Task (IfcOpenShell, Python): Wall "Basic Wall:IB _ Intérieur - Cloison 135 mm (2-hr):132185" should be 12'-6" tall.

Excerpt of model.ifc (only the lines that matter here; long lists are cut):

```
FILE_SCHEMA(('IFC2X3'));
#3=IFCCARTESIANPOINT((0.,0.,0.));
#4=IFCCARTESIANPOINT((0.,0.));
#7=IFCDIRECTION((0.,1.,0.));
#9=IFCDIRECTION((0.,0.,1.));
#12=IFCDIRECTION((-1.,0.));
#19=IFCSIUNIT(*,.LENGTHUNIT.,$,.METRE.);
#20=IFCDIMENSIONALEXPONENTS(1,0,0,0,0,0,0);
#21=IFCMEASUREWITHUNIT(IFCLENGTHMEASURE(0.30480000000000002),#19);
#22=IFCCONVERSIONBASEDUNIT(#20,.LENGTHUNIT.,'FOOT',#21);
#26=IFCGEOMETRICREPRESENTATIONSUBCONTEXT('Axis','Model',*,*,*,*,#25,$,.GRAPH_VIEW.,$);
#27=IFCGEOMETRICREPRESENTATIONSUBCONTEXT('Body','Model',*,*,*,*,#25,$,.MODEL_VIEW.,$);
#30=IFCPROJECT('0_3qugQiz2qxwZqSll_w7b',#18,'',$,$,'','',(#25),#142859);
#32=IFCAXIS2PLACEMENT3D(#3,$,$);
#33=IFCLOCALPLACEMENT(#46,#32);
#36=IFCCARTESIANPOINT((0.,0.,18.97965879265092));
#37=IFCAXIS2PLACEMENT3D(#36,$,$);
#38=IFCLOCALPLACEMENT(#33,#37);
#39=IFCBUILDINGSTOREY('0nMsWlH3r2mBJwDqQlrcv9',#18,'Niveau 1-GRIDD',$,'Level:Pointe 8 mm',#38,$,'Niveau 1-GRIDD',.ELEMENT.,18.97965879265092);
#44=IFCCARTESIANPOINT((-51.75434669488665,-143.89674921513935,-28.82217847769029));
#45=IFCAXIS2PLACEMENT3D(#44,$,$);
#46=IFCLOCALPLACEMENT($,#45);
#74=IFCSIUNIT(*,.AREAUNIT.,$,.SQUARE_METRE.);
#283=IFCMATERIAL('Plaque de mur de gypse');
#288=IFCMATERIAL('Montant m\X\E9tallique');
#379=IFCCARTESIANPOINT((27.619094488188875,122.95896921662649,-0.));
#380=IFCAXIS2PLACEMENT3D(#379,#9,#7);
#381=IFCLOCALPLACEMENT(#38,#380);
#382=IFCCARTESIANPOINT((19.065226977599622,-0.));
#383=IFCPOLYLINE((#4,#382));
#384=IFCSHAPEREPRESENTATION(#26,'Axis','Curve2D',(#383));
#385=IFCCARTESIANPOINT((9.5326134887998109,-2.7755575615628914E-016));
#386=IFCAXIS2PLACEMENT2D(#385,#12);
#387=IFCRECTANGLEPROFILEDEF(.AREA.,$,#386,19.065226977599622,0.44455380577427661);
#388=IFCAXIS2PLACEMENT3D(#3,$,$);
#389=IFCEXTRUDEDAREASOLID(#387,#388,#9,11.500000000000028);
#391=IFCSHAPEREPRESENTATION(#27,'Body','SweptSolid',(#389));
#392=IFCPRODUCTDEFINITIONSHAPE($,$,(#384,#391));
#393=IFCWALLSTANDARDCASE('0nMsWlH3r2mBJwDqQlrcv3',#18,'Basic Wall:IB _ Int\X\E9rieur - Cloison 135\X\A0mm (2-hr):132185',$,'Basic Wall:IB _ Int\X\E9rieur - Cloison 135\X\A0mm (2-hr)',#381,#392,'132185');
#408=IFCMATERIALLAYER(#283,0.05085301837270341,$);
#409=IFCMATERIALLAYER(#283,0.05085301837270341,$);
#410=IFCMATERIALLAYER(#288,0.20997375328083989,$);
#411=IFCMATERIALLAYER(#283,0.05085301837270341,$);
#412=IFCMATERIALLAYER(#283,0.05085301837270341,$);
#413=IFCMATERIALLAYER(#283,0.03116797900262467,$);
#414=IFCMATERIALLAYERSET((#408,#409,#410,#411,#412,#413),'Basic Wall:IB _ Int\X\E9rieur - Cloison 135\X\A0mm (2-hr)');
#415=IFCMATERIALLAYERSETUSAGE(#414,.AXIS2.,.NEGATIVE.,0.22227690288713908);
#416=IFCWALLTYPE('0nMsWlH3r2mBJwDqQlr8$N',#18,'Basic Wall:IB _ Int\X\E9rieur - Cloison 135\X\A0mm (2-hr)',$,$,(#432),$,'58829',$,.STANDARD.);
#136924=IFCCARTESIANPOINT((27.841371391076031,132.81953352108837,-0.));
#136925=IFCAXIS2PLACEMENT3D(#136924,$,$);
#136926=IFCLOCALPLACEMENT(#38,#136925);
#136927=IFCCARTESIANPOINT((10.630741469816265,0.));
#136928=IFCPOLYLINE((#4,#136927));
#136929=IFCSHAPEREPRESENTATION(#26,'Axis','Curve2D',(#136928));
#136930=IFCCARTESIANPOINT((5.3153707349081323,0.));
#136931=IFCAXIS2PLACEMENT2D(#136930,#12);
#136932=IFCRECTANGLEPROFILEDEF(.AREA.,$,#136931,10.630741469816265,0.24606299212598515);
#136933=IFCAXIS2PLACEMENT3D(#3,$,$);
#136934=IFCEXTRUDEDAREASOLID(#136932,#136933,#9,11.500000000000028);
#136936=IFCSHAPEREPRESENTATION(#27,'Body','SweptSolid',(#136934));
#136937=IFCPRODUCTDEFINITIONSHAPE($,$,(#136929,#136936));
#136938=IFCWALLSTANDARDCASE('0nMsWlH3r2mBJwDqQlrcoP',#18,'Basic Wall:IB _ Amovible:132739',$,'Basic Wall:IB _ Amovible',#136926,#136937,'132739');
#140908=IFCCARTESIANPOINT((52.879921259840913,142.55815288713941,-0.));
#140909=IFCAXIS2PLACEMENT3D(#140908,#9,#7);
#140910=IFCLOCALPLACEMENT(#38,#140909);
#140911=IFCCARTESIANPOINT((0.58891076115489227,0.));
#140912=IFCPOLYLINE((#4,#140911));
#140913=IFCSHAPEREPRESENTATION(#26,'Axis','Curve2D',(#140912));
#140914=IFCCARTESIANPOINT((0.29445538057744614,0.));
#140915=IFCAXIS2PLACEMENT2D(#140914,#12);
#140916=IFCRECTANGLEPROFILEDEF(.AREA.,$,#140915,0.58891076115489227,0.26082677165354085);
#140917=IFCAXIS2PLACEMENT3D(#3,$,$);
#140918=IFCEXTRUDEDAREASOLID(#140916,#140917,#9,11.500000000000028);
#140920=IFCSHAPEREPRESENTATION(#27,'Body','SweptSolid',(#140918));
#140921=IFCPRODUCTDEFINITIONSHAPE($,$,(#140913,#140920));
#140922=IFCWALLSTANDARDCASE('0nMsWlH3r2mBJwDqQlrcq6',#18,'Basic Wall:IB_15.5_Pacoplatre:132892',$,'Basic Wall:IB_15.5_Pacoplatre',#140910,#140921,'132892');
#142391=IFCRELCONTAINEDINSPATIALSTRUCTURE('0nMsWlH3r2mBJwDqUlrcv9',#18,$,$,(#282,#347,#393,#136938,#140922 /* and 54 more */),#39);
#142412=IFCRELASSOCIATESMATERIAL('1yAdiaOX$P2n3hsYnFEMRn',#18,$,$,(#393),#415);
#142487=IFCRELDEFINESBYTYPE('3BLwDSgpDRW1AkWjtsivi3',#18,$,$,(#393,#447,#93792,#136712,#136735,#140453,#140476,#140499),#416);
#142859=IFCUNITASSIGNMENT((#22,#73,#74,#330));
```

```python
import ifcopenshell
import ifcopenshell.geom
import ifcopenshell.util.representation
import ifcopenshell.util.shape
import ifcopenshell.util.unit

model = ifcopenshell.open("model.ifc")
unit_scale = ifcopenshell.util.unit.calculate_unit_scale(model)
settings = ifcopenshell.geom.settings()


def volume(element):
    """Net volume in cubic metres, openings subtracted."""
    shape = ifcopenshell.geom.create_shape(settings, element)
    return ifcopenshell.util.shape.get_volume(shape.geometry)


wall = model.by_guid("0nMsWlH3r2mBJwDqQlrcv3")
before = volume(wall)

body = ifcopenshell.util.representation.get_representation(wall, "Model", "Body")
solid = body.Items[0]
old_height = solid.Depth
solid.Depth = 150 * 0.0254 / unit_scale
after = volume(wall)

print(f"height {old_height:g} -> {solid.Depth:g}, volume {before:.3f} -> {after:.3f} m3")

model.write("model_v2.ifc")
```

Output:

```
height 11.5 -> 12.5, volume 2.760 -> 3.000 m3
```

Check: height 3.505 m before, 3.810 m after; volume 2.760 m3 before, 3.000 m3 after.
